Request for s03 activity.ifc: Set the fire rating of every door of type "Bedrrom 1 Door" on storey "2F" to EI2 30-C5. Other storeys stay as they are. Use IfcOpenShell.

First a look at what the model holds.

```python
import ifcopenshell
import ifcopenshell.util.element

model = ifcopenshell.open("s03 activity.ifc")
print(model.schema)
storey = next(s for s in model.by_type("IfcBuildingStorey") if s.Name == "2F")
doors = [e for e in ifcopenshell.util.element.get_decomposition(storey) if e.is_a("IfcDoor")]
seen = {}
for e in doors:
    element_type = ifcopenshell.util.element.get_type(e)
    key = (element_type.Name if element_type != e and element_type else None, ifcopenshell.util.element.get_pset(e, "Pset_DoorCommon", "FireRating"))
    seen[key] = seen.get(key, 0) + 1
for (name, value), count in sorted(seen.items(), key=str):
    print(count, "x", name, "|", value)
```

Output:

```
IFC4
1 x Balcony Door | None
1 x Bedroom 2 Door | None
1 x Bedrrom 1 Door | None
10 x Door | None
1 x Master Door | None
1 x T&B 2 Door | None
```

```python
import ifcopenshell
import ifcopenshell.api.pset
import ifcopenshell.util.element

model = ifcopenshell.open("s03 activity.ifc")

storey = next(s for s in model.by_type("IfcBuildingStorey") if s.Name == "2F")
doors = [e for e in ifcopenshell.util.element.get_decomposition(storey) if e.is_a("IfcDoor")]

count = 0
for e in doors:
    element_type = ifcopenshell.util.element.get_type(e)
    if element_type in (None, e) or element_type.Name != "Bedrrom 1 Door":
        continue
    # add_pset returns the element's existing set when there is one.
    pset = ifcopenshell.api.pset.add_pset(model, product=e, name="Pset_DoorCommon")
    ifcopenshell.api.pset.edit_pset(model, pset=pset, properties={"FireRating": "EI2 30-C5"})
    count += 1

print(count, "doors updated")

model.write("s03 activity_edited.ifc")
```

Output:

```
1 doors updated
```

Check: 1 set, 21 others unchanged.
